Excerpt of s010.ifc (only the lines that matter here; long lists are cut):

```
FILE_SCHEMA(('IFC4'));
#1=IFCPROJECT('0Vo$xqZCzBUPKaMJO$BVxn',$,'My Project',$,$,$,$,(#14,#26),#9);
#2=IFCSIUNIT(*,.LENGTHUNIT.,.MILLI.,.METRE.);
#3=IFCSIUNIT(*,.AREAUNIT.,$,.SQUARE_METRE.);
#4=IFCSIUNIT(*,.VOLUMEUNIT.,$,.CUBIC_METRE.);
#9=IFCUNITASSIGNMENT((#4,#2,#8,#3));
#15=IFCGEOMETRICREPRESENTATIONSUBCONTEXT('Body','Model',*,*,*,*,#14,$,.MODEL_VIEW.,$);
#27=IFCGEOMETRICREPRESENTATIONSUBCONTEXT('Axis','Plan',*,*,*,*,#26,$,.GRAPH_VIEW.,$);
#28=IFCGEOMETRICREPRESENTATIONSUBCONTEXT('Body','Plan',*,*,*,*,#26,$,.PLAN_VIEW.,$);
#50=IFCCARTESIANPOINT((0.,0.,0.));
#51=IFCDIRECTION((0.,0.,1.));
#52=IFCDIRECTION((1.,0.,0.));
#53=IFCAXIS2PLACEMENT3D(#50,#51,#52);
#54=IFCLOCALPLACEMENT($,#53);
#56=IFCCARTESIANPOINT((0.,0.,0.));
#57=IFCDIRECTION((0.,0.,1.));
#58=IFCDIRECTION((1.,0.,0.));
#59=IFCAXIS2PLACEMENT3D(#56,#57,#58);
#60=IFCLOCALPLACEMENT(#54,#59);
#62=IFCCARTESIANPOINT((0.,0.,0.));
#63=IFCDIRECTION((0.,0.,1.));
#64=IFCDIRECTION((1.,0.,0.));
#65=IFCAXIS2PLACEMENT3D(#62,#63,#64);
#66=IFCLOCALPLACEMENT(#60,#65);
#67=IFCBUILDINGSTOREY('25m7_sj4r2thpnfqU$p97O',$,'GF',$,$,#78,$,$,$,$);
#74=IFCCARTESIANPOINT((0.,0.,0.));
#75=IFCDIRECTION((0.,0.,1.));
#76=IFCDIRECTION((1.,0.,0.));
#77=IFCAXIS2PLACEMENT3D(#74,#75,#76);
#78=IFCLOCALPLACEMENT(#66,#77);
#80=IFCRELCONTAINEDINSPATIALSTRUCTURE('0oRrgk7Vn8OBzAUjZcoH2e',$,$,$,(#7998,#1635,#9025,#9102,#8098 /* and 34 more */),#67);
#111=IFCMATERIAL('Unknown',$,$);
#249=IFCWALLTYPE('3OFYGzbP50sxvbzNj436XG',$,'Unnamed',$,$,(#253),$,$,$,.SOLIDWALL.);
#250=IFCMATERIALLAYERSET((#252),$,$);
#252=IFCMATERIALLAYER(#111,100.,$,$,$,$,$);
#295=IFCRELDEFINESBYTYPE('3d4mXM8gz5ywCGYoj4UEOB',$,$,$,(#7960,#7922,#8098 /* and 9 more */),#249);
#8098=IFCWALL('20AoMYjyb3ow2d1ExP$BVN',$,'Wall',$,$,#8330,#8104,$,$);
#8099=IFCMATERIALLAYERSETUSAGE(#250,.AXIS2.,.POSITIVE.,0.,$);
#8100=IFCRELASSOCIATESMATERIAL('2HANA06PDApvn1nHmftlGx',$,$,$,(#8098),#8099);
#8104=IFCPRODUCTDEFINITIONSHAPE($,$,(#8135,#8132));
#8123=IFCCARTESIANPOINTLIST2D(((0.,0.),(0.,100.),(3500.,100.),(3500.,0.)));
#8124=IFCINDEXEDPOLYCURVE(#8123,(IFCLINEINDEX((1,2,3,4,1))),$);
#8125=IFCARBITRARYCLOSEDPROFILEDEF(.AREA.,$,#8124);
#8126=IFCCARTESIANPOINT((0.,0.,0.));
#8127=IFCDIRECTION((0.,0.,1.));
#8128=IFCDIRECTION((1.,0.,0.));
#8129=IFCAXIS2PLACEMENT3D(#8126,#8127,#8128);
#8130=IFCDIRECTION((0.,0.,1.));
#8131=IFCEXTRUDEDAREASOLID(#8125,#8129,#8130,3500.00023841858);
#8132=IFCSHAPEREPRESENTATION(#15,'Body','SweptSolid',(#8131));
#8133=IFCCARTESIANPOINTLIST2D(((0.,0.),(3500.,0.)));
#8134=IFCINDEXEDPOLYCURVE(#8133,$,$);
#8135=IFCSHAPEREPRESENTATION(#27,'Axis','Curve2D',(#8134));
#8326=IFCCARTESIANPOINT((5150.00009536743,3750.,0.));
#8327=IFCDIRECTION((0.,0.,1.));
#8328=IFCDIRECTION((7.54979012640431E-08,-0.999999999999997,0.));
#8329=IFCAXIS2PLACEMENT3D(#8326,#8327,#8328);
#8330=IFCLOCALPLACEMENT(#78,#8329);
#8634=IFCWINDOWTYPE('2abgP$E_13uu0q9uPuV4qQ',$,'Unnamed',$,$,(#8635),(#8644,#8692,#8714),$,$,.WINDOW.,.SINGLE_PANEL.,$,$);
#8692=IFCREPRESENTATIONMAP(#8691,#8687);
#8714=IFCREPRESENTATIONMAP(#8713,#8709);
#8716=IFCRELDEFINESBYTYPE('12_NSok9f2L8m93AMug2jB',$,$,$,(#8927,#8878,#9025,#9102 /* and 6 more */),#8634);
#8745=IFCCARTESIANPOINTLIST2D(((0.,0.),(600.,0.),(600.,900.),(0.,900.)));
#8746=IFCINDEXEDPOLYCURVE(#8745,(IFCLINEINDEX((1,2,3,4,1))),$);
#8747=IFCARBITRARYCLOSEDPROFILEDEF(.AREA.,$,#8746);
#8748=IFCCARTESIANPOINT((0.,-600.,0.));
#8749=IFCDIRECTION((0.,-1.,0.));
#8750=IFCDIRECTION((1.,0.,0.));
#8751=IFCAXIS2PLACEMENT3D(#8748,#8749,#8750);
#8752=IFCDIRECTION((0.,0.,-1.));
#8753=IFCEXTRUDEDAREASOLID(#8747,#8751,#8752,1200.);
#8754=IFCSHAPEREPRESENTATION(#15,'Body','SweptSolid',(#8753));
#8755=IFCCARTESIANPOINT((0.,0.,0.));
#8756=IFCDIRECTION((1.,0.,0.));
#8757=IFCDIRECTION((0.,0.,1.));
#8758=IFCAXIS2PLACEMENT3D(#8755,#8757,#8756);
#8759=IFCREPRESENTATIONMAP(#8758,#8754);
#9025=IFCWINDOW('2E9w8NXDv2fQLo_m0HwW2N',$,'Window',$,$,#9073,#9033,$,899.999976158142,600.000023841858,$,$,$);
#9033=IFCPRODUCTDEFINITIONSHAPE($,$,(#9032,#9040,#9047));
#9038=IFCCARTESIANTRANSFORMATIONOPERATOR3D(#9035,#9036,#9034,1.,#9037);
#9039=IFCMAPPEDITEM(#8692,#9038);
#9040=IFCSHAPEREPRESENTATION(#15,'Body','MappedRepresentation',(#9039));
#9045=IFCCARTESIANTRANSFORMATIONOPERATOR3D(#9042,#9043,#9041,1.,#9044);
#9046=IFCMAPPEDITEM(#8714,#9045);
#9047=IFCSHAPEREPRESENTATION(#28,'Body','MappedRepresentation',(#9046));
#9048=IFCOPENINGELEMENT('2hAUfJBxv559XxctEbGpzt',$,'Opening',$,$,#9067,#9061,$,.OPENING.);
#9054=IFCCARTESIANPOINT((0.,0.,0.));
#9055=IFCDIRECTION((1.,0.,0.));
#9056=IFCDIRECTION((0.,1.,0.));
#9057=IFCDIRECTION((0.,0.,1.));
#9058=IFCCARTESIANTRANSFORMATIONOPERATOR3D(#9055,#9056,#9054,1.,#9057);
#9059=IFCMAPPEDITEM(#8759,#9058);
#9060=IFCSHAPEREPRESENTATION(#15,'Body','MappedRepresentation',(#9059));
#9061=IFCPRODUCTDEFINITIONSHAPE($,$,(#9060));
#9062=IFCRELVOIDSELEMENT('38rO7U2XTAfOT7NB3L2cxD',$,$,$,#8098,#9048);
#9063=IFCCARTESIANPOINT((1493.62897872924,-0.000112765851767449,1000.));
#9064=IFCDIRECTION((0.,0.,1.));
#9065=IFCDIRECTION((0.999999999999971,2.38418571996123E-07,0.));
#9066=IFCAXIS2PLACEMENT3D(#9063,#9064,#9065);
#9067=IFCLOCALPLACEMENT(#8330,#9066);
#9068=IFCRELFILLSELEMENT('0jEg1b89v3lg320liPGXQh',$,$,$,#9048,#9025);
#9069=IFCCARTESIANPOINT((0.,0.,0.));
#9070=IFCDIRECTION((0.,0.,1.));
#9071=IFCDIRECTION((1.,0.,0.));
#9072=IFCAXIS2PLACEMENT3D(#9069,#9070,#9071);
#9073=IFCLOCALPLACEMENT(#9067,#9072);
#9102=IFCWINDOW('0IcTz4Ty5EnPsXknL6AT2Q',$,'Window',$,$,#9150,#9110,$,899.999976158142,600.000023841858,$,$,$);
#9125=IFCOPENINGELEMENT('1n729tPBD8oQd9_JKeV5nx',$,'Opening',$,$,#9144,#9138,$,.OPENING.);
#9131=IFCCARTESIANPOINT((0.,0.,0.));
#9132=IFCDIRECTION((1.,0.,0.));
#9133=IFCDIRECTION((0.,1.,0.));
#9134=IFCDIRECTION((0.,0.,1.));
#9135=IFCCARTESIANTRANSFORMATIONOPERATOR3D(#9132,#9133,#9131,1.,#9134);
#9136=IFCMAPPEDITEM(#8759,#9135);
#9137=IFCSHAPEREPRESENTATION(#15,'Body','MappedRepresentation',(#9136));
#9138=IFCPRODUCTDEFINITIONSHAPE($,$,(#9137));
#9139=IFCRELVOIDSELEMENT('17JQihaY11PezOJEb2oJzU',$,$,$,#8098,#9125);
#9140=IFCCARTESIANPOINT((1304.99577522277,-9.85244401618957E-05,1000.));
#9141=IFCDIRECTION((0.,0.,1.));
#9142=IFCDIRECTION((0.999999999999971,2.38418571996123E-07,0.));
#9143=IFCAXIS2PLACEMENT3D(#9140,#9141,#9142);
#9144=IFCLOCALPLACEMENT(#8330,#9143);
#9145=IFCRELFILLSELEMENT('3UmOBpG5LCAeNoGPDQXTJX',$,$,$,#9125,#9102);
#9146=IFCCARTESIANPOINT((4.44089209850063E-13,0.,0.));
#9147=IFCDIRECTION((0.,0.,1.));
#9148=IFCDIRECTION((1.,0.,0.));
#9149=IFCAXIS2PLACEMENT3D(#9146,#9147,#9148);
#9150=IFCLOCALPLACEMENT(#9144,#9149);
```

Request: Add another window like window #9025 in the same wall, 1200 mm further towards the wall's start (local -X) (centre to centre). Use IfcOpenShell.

```python
import ifcopenshell
import ifcopenshell.api.feature
import ifcopenshell.api.geometry
import ifcopenshell.api.root
import ifcopenshell.geom
import ifcopenshell.util.element
import ifcopenshell.util.placement
import ifcopenshell.util.shape
import ifcopenshell.util.unit

model = ifcopenshell.open("s010.ifc")
unit_scale = ifcopenshell.util.unit.calculate_unit_scale(model)
settings = ifcopenshell.geom.settings()


def volume(element):
    """Net volume in cubic metres, openings subtracted."""
    shape = ifcopenshell.geom.create_shape(settings, element)
    return ifcopenshell.util.shape.get_volume(shape.geometry)


window = model.by_guid("2E9w8NXDv2fQLo_m0HwW2N")
opening = window.FillsVoids[0].RelatingOpeningElement
wall = opening.VoidsElements[0].RelatingBuildingElement
before = volume(wall)
shift = ifcopenshell.util.placement.get_local_placement(wall.ObjectPlacement)[:3, 0] * -1.2 / unit_scale

# copy_class copies the void relationship, type, container and properties, but no geometry.
new_opening = ifcopenshell.api.root.copy_class(model, product=opening)
new_opening.Representation = ifcopenshell.util.element.copy_deep(
    model, opening.Representation, exclude=["IfcGeometricRepresentationContext", "IfcRepresentationMap"]
)
new_window = ifcopenshell.api.root.copy_class(model, product=window)
new_window.Representation = ifcopenshell.util.element.copy_deep(
    model, window.Representation, exclude=["IfcGeometricRepresentationContext", "IfcRepresentationMap"]
)
ifcopenshell.api.feature.add_filling(model, opening=new_opening, element=new_window)

for old, new in ((opening, new_opening), (window, new_window)):
    matrix = ifcopenshell.util.placement.get_local_placement(old.ObjectPlacement)
    matrix[:3, 3] += shift
    ifcopenshell.api.geometry.edit_object_placement(model, product=new, matrix=matrix, is_si=False)

after = volume(wall)

print(f"wall volume {before:.3f} -> {after:.3f} m3")

model.write("s010_v2.ifc")
```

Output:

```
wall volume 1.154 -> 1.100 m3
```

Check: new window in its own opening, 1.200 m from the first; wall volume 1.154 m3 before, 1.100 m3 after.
